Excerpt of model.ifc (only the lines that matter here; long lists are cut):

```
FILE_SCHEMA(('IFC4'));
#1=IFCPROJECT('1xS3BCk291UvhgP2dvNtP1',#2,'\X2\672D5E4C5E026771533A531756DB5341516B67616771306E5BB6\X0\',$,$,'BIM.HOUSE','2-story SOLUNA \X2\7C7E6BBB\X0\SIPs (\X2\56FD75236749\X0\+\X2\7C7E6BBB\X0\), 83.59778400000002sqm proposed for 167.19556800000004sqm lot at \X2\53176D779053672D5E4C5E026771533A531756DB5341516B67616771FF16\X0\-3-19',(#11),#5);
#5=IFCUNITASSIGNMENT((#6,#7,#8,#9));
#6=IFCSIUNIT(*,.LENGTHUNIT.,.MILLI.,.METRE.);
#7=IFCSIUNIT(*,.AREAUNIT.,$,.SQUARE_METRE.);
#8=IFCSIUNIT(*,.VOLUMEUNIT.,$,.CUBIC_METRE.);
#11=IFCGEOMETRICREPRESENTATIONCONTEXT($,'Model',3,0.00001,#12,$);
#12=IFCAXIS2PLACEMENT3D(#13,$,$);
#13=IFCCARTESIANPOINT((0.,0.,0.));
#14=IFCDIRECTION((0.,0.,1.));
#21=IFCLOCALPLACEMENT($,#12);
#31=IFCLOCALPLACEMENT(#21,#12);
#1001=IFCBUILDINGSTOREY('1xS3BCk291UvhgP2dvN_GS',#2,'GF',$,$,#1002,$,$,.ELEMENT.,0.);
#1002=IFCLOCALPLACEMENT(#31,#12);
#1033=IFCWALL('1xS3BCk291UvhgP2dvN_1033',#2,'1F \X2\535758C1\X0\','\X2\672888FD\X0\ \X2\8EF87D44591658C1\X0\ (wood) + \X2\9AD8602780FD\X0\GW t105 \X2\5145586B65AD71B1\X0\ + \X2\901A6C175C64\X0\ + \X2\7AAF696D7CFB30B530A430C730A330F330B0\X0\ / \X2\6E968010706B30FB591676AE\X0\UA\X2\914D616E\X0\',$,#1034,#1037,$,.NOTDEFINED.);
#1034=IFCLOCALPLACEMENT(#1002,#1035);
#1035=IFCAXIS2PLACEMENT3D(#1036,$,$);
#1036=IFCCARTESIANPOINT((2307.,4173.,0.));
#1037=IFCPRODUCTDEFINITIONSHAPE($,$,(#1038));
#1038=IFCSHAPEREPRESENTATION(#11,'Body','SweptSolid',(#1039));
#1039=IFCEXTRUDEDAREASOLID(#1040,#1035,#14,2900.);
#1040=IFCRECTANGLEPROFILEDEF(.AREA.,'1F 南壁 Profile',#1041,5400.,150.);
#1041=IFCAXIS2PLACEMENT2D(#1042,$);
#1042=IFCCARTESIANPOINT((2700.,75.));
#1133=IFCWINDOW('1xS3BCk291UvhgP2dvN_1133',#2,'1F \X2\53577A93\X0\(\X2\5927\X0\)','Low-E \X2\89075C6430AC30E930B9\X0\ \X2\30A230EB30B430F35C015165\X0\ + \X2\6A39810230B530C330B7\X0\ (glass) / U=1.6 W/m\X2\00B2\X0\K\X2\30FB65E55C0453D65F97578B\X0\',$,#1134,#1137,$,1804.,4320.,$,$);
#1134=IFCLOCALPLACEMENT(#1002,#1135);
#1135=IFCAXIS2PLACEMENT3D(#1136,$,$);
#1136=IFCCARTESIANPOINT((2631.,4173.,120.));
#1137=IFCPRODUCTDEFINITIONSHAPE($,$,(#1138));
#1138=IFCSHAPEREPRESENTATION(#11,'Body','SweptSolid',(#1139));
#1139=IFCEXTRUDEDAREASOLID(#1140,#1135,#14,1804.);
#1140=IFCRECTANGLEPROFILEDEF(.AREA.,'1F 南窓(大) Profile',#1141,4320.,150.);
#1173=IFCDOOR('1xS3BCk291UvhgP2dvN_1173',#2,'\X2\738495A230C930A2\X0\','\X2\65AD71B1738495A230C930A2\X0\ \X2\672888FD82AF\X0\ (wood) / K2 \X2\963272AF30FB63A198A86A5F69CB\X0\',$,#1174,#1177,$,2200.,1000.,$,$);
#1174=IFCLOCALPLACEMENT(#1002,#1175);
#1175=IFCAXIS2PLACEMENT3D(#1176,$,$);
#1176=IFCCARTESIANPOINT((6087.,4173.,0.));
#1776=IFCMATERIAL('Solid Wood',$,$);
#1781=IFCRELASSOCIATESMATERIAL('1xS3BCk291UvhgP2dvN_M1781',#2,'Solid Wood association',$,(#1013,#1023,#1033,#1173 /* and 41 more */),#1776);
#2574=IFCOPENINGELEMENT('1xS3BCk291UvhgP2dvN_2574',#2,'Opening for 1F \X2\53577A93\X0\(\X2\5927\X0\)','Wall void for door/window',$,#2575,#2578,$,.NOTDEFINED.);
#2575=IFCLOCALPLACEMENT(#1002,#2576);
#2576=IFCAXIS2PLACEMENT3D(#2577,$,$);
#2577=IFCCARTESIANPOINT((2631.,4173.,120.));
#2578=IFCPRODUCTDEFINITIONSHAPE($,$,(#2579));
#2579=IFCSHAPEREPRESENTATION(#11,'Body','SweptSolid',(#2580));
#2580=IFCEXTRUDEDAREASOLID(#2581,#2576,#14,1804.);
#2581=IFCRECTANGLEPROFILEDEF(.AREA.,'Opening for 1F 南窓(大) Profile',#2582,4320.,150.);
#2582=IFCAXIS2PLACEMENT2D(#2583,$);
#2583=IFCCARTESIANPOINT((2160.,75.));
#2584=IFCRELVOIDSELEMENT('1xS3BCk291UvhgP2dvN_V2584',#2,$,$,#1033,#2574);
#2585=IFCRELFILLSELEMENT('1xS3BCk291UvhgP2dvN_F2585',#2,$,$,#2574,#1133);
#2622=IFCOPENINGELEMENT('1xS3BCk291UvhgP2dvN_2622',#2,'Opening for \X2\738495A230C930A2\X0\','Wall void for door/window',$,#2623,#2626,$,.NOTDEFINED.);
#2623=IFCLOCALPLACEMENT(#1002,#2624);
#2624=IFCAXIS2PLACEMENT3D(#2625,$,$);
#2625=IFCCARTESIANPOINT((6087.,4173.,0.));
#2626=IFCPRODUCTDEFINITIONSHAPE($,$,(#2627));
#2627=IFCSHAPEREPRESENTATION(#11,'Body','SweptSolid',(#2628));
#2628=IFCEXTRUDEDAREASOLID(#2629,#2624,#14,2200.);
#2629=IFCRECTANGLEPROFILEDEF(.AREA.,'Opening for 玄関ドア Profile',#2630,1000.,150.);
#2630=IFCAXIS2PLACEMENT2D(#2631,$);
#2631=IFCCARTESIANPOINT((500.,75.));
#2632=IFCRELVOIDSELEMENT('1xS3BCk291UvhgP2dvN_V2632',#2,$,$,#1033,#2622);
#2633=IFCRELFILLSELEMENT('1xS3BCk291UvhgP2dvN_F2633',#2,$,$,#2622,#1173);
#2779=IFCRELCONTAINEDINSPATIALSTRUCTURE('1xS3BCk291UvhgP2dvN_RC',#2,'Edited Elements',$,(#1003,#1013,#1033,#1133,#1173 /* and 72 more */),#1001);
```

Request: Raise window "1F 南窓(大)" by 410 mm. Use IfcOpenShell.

```python
import numpy as np
import ifcopenshell
import ifcopenshell.api.geometry
import ifcopenshell.util.placement
import ifcopenshell.util.unit

model = ifcopenshell.open("model.ifc")
unit_scale = ifcopenshell.util.unit.calculate_unit_scale(model)

window = model.by_id(1133)
opening = window.FillsVoids[0].RelatingOpeningElement
dz = 410.0

shift = np.array([0.0, 0.0, dz])
# The window is not placed relative to its opening, so move both.
for product in (opening, window):
    matrix = ifcopenshell.util.placement.get_local_placement(product.ObjectPlacement)
    matrix[:3, 3] += shift
    ifcopenshell.api.geometry.edit_object_placement(model, product=product, matrix=matrix, is_si=False)

print(f"moved by {dz * unit_scale:+.3f} m")

model.write("model_edited.ifc")
```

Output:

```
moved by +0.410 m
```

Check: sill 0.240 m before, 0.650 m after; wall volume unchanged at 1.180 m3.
